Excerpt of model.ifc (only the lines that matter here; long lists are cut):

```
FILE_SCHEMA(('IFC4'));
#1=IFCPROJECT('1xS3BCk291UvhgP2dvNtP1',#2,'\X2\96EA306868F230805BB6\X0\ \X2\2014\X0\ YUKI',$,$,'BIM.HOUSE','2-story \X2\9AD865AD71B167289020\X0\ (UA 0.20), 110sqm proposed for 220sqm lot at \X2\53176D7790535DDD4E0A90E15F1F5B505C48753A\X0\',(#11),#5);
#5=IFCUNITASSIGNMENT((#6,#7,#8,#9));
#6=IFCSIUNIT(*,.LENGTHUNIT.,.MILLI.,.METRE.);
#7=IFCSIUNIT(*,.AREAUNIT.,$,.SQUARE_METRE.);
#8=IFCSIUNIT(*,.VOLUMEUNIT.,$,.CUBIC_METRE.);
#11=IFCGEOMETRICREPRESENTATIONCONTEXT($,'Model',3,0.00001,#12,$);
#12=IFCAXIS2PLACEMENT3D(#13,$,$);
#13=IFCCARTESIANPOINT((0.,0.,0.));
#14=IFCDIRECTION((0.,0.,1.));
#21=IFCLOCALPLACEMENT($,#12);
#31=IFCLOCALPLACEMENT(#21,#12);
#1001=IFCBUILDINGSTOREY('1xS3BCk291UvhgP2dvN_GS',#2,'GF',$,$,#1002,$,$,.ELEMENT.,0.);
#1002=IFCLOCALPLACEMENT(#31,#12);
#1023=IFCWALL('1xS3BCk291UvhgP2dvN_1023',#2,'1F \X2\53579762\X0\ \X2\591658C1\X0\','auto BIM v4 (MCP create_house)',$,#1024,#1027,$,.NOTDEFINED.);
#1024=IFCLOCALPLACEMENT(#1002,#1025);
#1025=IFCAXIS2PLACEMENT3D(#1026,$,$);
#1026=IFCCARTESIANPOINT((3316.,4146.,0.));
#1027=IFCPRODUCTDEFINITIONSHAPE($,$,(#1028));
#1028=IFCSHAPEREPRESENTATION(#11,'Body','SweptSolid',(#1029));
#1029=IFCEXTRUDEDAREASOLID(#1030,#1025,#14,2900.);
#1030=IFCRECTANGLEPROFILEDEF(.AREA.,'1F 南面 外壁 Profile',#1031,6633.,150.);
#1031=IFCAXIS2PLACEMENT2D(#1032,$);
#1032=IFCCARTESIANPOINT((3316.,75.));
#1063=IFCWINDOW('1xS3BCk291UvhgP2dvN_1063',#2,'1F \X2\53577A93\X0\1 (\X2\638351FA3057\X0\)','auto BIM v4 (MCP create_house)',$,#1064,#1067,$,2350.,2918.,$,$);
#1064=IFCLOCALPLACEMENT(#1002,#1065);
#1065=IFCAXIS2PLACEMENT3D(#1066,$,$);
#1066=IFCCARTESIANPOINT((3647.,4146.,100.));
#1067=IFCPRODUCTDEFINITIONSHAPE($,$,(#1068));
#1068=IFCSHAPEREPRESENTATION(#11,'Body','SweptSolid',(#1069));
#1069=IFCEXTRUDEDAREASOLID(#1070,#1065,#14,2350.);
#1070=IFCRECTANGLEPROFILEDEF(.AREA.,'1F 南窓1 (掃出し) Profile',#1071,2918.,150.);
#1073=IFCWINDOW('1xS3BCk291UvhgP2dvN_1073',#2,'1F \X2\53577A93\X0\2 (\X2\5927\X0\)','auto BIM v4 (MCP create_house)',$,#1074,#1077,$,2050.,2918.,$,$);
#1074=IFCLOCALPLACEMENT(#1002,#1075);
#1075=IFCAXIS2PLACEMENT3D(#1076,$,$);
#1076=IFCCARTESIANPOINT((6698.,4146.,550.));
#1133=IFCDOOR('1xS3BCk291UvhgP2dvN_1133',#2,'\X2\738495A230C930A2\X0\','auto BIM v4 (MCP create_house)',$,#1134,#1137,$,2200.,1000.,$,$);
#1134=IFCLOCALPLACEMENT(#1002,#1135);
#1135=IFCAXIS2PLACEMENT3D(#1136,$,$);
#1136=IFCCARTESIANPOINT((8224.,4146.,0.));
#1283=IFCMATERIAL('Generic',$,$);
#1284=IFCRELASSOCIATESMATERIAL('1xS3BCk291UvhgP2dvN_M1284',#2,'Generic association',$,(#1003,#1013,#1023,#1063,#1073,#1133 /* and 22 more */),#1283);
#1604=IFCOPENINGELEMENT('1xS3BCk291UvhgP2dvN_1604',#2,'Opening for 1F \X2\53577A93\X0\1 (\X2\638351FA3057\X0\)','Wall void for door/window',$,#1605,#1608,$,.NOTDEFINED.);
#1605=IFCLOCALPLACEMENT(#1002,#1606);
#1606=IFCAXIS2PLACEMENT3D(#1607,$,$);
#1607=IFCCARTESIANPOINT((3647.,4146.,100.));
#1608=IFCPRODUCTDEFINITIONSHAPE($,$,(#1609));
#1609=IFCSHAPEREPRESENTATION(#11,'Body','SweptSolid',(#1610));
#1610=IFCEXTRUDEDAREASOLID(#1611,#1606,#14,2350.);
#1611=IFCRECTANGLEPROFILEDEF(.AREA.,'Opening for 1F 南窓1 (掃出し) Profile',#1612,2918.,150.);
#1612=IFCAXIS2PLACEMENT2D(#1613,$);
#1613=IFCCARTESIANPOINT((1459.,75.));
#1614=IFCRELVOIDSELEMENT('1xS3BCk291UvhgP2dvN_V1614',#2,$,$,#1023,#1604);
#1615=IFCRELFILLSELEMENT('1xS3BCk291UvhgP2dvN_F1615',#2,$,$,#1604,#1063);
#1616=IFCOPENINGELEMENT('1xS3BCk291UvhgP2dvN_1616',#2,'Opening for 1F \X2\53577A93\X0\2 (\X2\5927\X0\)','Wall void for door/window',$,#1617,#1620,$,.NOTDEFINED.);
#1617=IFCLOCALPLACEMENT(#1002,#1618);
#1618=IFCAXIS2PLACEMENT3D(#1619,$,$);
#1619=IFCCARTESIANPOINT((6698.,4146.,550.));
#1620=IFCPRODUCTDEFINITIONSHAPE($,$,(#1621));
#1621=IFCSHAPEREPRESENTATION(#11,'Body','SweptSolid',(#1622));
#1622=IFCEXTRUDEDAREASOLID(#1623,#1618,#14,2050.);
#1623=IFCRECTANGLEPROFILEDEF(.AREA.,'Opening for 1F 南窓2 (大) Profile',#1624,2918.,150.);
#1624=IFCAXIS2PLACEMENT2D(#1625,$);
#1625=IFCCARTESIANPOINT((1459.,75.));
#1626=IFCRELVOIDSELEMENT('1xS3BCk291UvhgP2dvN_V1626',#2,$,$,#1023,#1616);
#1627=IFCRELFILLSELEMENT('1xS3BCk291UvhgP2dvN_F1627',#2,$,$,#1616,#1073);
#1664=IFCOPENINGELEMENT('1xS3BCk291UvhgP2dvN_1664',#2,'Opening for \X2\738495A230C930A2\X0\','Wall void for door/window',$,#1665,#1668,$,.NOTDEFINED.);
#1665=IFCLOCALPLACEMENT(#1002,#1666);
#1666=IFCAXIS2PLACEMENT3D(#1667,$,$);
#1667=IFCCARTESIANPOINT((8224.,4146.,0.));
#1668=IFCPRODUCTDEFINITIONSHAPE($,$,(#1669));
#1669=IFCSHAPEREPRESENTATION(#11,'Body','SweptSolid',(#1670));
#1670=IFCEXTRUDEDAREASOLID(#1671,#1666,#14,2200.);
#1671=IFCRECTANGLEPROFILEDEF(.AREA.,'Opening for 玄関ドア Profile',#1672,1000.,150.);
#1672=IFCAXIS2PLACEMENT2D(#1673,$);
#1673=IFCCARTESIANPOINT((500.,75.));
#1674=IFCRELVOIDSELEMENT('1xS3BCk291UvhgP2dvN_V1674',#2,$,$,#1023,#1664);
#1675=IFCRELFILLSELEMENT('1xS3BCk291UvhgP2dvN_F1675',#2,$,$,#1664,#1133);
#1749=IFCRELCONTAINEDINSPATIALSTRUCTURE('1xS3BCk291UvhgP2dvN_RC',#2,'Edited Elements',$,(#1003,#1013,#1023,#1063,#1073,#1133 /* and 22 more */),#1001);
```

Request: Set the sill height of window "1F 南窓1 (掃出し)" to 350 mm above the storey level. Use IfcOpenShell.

```python
import numpy as np
import ifcopenshell
import ifcopenshell.api.geometry
import ifcopenshell.geom
import ifcopenshell.util.element
import ifcopenshell.util.placement
import ifcopenshell.util.shape
import ifcopenshell.util.unit

model = ifcopenshell.open("model.ifc")
unit_scale = ifcopenshell.util.unit.calculate_unit_scale(model)

window = model.by_guid("1xS3BCk291UvhgP2dvN_1063")
opening = window.FillsVoids[0].RelatingOpeningElement
storey = ifcopenshell.util.element.get_container(window, ifc_class="IfcBuildingStorey")
level = ifcopenshell.util.placement.get_local_placement(storey.ObjectPlacement)[2, 3]

# The opening's origin need not be at the sill, so measure its lowest point.
shape = ifcopenshell.geom.create_shape(ifcopenshell.geom.settings(), opening)
bottom = ifcopenshell.util.shape.get_shape_bottom_elevation(shape, shape.geometry) / unit_scale
dz = level + 350.0 - bottom

shift = np.array([0.0, 0.0, dz])
# The window is not placed relative to its opening, so move both.
for product in (opening, window):
    matrix = ifcopenshell.util.placement.get_local_placement(product.ObjectPlacement)
    matrix[:3, 3] += shift
    ifcopenshell.api.geometry.edit_object_placement(model, product=product, matrix=matrix, is_si=False)

print(f"moved by {dz * unit_scale:+.3f} m")

model.write("model_rev.ifc")
```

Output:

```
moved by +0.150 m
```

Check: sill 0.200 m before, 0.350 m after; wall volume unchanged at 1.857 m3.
